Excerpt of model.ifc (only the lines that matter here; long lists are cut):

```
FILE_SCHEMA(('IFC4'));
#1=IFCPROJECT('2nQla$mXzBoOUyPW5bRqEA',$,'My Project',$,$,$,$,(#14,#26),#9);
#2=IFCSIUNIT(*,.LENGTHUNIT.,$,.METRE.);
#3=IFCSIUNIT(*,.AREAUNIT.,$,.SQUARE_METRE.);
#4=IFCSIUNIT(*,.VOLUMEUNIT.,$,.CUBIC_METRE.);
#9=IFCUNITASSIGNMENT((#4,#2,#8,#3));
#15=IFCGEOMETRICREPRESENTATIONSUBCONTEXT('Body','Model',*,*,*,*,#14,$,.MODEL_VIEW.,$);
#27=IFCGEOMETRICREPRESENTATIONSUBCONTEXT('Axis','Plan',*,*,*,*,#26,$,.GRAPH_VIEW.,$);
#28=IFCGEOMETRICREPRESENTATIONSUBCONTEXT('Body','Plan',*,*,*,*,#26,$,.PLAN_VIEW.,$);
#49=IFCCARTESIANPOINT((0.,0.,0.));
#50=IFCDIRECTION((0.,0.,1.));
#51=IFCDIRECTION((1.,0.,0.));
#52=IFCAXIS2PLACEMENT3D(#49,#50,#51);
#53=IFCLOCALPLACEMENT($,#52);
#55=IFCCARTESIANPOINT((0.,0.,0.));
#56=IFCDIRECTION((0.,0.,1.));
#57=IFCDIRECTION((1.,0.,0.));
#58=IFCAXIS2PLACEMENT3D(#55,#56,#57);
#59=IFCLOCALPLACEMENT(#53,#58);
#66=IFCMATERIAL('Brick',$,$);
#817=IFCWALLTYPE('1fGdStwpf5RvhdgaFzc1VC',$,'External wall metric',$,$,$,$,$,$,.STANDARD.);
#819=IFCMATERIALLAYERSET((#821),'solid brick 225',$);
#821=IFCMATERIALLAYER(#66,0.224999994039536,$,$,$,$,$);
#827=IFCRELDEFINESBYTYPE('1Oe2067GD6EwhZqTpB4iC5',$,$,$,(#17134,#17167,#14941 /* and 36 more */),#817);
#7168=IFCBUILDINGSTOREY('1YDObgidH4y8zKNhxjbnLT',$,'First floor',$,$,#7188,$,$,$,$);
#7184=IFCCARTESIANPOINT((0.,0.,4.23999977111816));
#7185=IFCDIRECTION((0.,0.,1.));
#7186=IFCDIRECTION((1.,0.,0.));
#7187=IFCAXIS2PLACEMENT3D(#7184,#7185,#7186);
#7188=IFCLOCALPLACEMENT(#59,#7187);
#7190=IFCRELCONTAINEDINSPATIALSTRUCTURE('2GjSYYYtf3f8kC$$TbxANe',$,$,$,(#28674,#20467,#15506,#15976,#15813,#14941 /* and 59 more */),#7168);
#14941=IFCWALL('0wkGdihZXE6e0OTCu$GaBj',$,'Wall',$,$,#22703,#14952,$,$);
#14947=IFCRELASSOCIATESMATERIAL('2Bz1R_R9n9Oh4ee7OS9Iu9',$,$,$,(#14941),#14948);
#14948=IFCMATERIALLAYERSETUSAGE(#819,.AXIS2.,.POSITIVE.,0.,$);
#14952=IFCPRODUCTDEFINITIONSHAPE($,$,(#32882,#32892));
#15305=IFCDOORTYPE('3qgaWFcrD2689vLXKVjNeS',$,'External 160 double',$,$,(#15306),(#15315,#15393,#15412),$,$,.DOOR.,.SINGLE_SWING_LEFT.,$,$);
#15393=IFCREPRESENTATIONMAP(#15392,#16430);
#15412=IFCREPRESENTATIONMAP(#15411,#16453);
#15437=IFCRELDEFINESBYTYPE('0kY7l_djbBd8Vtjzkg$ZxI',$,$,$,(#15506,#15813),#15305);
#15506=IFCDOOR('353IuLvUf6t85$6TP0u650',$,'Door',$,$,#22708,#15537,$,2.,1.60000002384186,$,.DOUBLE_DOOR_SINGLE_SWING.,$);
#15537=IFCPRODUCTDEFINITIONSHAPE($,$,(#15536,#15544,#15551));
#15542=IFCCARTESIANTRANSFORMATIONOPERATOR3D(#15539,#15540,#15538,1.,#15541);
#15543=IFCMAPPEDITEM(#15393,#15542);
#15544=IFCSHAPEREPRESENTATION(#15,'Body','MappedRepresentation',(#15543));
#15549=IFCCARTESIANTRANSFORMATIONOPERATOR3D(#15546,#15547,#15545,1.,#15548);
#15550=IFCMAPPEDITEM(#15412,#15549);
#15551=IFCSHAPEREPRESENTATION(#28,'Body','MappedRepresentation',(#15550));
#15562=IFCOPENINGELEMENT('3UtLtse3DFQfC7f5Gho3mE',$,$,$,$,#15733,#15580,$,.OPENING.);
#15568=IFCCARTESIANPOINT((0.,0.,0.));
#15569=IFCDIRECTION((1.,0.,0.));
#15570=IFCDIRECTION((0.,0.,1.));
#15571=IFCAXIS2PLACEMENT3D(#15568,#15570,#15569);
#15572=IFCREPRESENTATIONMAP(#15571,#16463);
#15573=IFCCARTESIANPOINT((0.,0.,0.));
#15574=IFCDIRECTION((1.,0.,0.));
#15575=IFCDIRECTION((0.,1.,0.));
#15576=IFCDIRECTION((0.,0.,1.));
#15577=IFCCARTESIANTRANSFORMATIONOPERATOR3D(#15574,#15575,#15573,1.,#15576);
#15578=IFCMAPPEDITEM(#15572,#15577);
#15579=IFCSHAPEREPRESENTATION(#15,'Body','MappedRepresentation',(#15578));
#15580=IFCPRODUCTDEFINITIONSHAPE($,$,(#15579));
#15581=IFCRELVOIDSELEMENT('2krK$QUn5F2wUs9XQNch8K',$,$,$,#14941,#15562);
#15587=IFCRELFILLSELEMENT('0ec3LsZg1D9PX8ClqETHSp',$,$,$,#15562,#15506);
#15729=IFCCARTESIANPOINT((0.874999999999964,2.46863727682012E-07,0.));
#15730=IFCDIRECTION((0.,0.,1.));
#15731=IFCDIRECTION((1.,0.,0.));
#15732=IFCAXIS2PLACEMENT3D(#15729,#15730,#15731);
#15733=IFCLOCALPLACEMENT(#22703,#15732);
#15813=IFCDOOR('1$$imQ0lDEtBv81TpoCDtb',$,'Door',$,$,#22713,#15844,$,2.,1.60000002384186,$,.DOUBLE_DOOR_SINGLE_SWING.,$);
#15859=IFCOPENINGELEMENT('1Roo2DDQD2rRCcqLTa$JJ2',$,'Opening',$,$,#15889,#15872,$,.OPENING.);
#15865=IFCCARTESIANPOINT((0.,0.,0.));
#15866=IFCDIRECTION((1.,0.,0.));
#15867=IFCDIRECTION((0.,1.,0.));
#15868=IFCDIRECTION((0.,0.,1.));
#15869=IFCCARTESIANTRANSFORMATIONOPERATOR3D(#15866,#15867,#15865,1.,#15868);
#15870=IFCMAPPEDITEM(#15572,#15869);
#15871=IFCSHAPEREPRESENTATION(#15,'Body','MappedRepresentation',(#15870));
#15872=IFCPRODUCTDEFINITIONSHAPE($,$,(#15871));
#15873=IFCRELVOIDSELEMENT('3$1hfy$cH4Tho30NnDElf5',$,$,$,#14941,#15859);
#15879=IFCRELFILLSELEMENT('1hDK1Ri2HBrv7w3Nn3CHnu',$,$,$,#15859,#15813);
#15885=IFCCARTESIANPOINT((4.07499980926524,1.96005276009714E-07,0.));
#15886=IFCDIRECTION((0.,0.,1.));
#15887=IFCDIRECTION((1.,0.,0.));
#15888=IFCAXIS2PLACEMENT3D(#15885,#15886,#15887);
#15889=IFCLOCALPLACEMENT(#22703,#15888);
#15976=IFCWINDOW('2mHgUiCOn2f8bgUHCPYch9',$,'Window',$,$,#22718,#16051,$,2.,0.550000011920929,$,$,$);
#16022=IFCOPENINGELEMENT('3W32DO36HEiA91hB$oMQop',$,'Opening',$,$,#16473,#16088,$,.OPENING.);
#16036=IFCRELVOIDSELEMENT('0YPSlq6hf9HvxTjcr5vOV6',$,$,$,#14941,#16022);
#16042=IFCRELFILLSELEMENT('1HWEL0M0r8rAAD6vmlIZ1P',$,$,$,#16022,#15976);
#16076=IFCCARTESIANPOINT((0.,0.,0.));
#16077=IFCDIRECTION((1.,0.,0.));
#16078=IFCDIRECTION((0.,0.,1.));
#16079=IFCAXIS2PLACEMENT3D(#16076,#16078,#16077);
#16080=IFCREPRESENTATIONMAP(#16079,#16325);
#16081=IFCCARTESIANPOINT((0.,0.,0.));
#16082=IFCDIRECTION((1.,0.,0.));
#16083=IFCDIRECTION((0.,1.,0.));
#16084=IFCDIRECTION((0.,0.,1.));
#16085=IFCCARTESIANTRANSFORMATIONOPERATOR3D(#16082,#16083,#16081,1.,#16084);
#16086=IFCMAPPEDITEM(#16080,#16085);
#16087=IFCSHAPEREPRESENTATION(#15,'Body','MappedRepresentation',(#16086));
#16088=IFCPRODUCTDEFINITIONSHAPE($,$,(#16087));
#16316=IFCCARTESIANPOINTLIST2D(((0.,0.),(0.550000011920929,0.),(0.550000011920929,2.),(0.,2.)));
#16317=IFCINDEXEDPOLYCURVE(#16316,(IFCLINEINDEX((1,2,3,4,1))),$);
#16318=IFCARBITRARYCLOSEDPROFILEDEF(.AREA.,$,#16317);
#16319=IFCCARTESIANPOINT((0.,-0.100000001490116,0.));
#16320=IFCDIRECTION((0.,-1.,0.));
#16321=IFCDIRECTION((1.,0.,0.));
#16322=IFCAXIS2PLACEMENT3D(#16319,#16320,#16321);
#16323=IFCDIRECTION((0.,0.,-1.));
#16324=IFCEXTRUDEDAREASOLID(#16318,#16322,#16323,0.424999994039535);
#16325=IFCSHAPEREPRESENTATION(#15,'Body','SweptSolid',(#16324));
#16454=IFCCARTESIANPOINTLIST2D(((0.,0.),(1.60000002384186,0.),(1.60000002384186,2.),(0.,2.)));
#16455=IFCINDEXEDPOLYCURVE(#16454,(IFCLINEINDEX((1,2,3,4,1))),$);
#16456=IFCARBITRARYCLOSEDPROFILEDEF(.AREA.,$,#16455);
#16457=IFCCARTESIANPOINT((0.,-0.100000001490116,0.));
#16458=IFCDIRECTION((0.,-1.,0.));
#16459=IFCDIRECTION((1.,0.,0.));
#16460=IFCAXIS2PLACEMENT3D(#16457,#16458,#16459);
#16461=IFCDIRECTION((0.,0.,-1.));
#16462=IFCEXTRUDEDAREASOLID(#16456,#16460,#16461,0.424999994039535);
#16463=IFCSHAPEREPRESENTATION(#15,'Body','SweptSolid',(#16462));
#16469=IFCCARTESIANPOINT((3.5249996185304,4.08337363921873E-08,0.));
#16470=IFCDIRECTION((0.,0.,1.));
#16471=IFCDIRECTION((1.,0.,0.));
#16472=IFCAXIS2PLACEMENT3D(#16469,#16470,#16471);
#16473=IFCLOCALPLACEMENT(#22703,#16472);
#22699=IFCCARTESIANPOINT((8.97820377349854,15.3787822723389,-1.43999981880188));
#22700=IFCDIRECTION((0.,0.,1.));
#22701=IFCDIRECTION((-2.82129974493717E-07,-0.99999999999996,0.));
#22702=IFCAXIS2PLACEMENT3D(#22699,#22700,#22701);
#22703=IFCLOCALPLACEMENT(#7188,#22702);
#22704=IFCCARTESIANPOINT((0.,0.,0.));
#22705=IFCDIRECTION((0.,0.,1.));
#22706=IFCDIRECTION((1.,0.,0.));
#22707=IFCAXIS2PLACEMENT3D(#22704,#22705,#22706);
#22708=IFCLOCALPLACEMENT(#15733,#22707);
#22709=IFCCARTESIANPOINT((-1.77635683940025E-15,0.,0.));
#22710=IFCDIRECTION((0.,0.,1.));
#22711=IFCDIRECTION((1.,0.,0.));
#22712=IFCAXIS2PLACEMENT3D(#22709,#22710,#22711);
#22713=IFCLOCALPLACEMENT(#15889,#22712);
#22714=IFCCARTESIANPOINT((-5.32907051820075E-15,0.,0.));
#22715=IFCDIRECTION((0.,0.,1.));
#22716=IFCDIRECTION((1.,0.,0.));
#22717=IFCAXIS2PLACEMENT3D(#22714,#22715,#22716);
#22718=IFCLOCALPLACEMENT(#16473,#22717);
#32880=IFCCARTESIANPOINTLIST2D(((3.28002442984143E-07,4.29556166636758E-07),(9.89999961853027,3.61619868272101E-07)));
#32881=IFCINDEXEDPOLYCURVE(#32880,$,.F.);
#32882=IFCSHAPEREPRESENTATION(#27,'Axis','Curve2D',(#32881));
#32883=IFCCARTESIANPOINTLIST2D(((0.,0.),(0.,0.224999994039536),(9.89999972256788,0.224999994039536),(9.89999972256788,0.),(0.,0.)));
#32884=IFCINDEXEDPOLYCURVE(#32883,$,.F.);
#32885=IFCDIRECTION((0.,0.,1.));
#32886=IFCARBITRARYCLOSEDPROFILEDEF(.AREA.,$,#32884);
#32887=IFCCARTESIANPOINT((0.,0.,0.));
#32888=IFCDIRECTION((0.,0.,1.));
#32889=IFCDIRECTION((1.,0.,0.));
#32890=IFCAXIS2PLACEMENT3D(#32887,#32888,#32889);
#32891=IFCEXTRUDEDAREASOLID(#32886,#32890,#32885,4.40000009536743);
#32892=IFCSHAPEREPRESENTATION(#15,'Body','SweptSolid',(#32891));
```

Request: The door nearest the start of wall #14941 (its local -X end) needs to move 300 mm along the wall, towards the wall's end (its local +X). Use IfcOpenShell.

```python
import ifcopenshell
import ifcopenshell.api.geometry
import ifcopenshell.util.placement
import ifcopenshell.util.unit

model = ifcopenshell.open("model.ifc")
unit_scale = ifcopenshell.util.unit.calculate_unit_scale(model)

door = model.by_guid("353IuLvUf6t85$6TP0u650")
opening = door.FillsVoids[0].RelatingOpeningElement
wall = opening.VoidsElements[0].RelatingBuildingElement

wall_matrix = ifcopenshell.util.placement.get_local_placement(wall.ObjectPlacement)
shift = wall_matrix[:3, 0] * 0.3 / unit_scale
before = ifcopenshell.util.placement.get_local_placement(door.ObjectPlacement)[:3, 3].copy()

# The door is placed relative to its opening, so it follows when the opening moves.
matrix = ifcopenshell.util.placement.get_local_placement(opening.ObjectPlacement)
matrix[:3, 3] += shift
ifcopenshell.api.geometry.edit_object_placement(
    model, product=opening, matrix=matrix, is_si=False, should_transform_children=True
)

after = ifcopenshell.util.placement.get_local_placement(door.ObjectPlacement)[:3, 3]
print("door moved by", (after - before).round(3) + 0.0)

model.write("model-out.ifc")
```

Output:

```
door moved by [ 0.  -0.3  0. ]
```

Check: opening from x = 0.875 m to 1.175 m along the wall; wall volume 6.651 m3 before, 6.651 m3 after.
